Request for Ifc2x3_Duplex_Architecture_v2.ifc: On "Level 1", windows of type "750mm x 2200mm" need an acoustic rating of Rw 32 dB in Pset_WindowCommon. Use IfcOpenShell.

First a look at what the model holds.

```python
import ifcopenshell
import ifcopenshell.util.element

model = ifcopenshell.open("Ifc2x3_Duplex_Architecture_v2.ifc")
print(model.schema)
storey = next(s for s in model.by_type("IfcBuildingStorey") if s.Name == "Level 1")
windows = [e for e in ifcopenshell.util.element.get_decomposition(storey) if e.is_a("IfcWindow")]
seen = {}
for e in windows:
    element_type = ifcopenshell.util.element.get_type(e)
    key = (element_type.Name if element_type != e and element_type else None, ifcopenshell.util.element.get_pset(e, "Pset_WindowCommon", "AcousticRating"))
    seen[key] = seen.get(key, 0) + 1
for (name, value), count in sorted(seen.items(), key=str):
    print(count, "x", name, "|", value)
```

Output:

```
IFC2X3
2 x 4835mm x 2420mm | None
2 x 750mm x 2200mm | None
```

```python
import ifcopenshell
import ifcopenshell.api.pset
import ifcopenshell.util.element

model = ifcopenshell.open("Ifc2x3_Duplex_Architecture_v2.ifc")

storey = next(s for s in model.by_type("IfcBuildingStorey") if s.Name == "Level 1")
windows = [e for e in ifcopenshell.util.element.get_decomposition(storey) if e.is_a("IfcWindow")]

count = 0
for e in windows:
    element_type = ifcopenshell.util.element.get_type(e)
    if element_type in (None, e) or element_type.Name != "750mm x 2200mm":
        continue
    # add_pset returns the element's existing set when there is one.
    pset = ifcopenshell.api.pset.add_pset(model, product=e, name="Pset_WindowCommon")
    ifcopenshell.api.pset.edit_pset(model, pset=pset, properties={"AcousticRating": "Rw 32 dB"})
    count += 1

print(count, "windows updated")

model.write("Ifc2x3_Duplex_Architecture_v2_edited.ifc")
```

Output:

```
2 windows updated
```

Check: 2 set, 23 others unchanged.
